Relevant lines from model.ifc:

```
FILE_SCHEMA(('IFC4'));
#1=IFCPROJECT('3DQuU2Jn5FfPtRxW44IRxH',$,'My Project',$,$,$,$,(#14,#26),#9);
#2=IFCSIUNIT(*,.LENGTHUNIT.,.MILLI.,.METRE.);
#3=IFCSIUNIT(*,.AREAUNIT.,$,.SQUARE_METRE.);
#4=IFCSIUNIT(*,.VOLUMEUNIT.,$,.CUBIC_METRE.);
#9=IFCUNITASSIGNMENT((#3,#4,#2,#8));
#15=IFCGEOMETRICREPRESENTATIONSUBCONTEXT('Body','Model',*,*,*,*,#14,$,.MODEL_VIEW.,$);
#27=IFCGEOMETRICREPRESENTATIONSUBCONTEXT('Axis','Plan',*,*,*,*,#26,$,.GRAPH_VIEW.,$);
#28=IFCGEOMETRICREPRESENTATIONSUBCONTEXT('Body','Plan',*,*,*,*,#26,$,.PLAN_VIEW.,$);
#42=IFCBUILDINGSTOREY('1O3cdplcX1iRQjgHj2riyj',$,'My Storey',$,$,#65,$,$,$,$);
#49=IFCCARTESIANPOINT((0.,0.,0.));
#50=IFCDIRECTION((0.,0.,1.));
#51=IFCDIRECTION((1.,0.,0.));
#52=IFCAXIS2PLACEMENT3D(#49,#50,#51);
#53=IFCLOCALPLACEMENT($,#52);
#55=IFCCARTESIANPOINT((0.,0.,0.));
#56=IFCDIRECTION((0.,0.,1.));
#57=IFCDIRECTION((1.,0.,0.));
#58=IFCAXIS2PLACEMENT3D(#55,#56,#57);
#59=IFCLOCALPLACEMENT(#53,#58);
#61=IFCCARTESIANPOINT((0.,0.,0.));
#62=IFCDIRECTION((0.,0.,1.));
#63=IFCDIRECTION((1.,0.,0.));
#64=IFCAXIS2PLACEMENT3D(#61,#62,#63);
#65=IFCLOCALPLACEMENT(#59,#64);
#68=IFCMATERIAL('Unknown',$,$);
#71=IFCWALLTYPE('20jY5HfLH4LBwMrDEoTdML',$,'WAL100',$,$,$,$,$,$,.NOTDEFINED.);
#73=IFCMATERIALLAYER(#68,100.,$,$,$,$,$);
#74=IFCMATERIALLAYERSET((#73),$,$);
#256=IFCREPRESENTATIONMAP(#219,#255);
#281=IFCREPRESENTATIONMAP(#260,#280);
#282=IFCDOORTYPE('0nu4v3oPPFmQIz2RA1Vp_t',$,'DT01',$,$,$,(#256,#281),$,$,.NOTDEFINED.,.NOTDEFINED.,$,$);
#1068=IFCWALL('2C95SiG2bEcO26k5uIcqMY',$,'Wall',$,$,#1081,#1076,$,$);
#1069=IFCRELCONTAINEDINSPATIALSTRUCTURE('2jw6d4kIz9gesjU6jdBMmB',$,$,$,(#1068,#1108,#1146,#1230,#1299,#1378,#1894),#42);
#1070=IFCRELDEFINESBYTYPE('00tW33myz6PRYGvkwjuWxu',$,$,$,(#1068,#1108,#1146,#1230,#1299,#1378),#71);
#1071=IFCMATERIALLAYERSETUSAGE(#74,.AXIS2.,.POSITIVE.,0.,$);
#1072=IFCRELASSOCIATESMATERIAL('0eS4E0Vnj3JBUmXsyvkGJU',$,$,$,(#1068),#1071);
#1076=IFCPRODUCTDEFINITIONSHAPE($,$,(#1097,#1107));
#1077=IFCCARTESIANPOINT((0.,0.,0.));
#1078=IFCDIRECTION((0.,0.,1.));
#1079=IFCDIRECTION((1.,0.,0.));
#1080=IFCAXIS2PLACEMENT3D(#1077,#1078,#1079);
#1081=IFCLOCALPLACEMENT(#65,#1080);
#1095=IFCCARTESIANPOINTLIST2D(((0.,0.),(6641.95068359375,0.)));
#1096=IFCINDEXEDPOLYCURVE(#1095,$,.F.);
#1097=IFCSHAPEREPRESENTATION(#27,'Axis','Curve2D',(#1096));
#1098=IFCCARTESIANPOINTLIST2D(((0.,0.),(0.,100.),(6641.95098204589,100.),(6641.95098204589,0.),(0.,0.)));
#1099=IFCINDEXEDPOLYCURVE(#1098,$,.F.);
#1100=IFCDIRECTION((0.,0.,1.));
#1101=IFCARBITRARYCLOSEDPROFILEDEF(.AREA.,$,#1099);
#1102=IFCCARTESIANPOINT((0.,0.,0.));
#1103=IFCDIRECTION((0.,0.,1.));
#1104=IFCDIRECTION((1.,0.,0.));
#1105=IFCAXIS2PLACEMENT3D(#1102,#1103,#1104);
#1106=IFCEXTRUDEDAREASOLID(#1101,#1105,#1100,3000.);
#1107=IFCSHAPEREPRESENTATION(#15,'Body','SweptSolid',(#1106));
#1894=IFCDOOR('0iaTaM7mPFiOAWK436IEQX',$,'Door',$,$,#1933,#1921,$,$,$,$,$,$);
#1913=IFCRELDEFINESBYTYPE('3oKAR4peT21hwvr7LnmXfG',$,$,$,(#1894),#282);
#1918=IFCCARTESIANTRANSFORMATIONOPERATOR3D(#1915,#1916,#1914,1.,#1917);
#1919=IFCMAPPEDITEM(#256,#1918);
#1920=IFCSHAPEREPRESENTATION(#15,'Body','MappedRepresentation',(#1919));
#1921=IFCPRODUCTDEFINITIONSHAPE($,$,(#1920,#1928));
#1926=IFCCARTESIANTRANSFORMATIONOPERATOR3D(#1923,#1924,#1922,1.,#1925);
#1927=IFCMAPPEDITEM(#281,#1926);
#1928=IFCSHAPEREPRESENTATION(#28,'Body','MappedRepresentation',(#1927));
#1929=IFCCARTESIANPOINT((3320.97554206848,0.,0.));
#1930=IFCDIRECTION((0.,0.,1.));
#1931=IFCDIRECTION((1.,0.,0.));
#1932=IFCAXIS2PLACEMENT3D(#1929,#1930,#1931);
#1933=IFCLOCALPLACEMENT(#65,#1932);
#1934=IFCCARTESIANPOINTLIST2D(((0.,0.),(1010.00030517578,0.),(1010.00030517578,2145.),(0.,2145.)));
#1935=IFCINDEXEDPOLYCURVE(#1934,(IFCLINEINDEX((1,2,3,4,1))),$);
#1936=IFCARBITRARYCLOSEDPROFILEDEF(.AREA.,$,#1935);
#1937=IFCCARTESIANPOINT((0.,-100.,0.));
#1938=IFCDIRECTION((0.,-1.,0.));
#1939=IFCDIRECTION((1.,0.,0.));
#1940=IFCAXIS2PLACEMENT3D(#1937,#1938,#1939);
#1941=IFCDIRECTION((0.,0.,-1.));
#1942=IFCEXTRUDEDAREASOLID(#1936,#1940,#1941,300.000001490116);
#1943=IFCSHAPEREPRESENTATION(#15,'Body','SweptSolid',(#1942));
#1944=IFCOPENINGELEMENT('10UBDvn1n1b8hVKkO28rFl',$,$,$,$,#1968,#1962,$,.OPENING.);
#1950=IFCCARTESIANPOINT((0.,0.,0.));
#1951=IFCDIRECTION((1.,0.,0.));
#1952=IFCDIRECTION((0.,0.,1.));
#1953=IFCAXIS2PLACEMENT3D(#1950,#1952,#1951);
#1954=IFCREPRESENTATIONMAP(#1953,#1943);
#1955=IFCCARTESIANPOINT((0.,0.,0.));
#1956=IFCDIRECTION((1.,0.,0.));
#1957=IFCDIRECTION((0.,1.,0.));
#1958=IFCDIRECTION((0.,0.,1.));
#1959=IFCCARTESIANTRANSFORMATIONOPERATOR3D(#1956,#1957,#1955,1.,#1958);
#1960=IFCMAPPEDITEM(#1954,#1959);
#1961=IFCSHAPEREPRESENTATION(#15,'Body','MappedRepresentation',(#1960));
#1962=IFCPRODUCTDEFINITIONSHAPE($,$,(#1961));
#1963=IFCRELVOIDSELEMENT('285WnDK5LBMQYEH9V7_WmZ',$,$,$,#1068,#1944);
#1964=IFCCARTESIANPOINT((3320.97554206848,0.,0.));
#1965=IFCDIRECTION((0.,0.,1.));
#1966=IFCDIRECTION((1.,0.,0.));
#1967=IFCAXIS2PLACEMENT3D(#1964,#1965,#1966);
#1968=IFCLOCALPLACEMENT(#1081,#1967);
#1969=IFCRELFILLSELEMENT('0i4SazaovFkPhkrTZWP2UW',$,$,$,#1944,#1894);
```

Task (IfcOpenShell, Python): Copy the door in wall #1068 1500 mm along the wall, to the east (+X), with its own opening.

```python
import ifcopenshell
import ifcopenshell.api.feature
import ifcopenshell.api.geometry
import ifcopenshell.api.root
import ifcopenshell.geom
import ifcopenshell.util.element
import ifcopenshell.util.placement
import ifcopenshell.util.shape
import ifcopenshell.util.unit

model = ifcopenshell.open("model.ifc")
unit_scale = ifcopenshell.util.unit.calculate_unit_scale(model)
settings = ifcopenshell.geom.settings()


def volume(element):
    """Net volume in cubic metres, openings subtracted."""
    shape = ifcopenshell.geom.create_shape(settings, element)
    return ifcopenshell.util.shape.get_volume(shape.geometry)


door = model.by_id(1894)
opening = door.FillsVoids[0].RelatingOpeningElement
wall = opening.VoidsElements[0].RelatingBuildingElement
before = volume(wall)
shift = ifcopenshell.util.placement.get_local_placement(wall.ObjectPlacement)[:3, 0] * 1.5 / unit_scale

# copy_class copies the void relationship, type, container and properties, but no geometry.
new_opening = ifcopenshell.api.root.copy_class(model, product=opening)
new_opening.Representation = ifcopenshell.util.element.copy_deep(
    model, opening.Representation, exclude=["IfcGeometricRepresentationContext", "IfcRepresentationMap"]
)
new_door = ifcopenshell.api.root.copy_class(model, product=door)
new_door.Representation = ifcopenshell.util.element.copy_deep(
    model, door.Representation, exclude=["IfcGeometricRepresentationContext", "IfcRepresentationMap"]
)
ifcopenshell.api.feature.add_filling(model, opening=new_opening, element=new_door)

for old, new in ((opening, new_opening), (door, new_door)):
    matrix = ifcopenshell.util.placement.get_local_placement(old.ObjectPlacement)
    matrix[:3, 3] += shift
    ifcopenshell.api.geometry.edit_object_placement(model, product=new, matrix=matrix, is_si=False)

after = volume(wall)

print(f"wall volume {before:.3f} -> {after:.3f} m3")

model.write("model_v2.ifc")
```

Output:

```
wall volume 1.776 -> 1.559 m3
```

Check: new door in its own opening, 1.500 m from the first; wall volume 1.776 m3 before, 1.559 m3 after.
